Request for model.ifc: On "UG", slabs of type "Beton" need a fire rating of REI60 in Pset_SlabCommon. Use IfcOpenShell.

First a look at what the model holds.

```python
import ifcopenshell
import ifcopenshell.util.element

model = ifcopenshell.open("model.ifc")
print(model.schema)
storey = next(s for s in model.by_type("IfcBuildingStorey") if s.Name == "UG")
slabs = [e for e in ifcopenshell.util.element.get_decomposition(storey) if e.is_a("IfcSlab")]
seen = {}
for e in slabs:
    element_type = ifcopenshell.util.element.get_type(e)
    key = (element_type.Name if element_type != e and element_type else None, ifcopenshell.util.element.get_pset(e, "Pset_SlabCommon", "FireRating"))
    seen[key] = seen.get(key, 0) + 1
for (name, value), count in sorted(seen.items(), key=str):
    print(count, "x", name, "|", value)
```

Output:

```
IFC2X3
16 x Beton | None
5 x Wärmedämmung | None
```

```python
import ifcopenshell
import ifcopenshell.api.pset
import ifcopenshell.util.element

model = ifcopenshell.open("model.ifc")

storey = next(s for s in model.by_type("IfcBuildingStorey") if s.Name == "UG")
slabs = [e for e in ifcopenshell.util.element.get_decomposition(storey) if e.is_a("IfcSlab")]

count = 0
for e in slabs:
    element_type = ifcopenshell.util.element.get_type(e)
    if element_type in (None, e) or element_type.Name != "Beton":
        continue
    # add_pset returns the element's existing set when there is one.
    pset = ifcopenshell.api.pset.add_pset(model, product=e, name="Pset_SlabCommon")
    ifcopenshell.api.pset.edit_pset(model, pset=pset, properties={"FireRating": "REI60"})
    count += 1

print(count, "slabs updated")

model.write("model_edited.ifc")
```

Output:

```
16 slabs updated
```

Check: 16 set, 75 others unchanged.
